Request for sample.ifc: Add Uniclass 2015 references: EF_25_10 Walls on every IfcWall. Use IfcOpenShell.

First a look at what the model holds.

```python
import ifcopenshell

model = ifcopenshell.open("sample.ifc")
print(model.schema)
print("classifications:", [c.Name for c in model.by_type("IfcClassification")])
for ifc_class in ("IfcDoor", "IfcRoof", "IfcStair", "IfcWall", "IfcWindow"):
    print(ifc_class, len(model.by_type(ifc_class)))
```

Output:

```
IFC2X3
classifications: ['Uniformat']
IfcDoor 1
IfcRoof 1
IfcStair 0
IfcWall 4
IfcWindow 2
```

```python
import ifcopenshell
import ifcopenshell.api.classification

model = ifcopenshell.open("sample.ifc")

# IFC2X3 requires Source and Edition and has no link from the project to the system.
system = model.create_entity("IfcClassification", Source="NBS", Edition="2015", Name="Uniclass 2015")

codes = {
    "IfcWall": ("EF_25_10", "Walls"),
}
for ifc_class, (code, name) in codes.items():
    products = model.by_type(ifc_class)
    ifcopenshell.api.classification.add_reference(
        model, products=products, classification=system, identification=code, name=name
    )
    print(code, len(products))

model.write("sample_v2.ifc")
```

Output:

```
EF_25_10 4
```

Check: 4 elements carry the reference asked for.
